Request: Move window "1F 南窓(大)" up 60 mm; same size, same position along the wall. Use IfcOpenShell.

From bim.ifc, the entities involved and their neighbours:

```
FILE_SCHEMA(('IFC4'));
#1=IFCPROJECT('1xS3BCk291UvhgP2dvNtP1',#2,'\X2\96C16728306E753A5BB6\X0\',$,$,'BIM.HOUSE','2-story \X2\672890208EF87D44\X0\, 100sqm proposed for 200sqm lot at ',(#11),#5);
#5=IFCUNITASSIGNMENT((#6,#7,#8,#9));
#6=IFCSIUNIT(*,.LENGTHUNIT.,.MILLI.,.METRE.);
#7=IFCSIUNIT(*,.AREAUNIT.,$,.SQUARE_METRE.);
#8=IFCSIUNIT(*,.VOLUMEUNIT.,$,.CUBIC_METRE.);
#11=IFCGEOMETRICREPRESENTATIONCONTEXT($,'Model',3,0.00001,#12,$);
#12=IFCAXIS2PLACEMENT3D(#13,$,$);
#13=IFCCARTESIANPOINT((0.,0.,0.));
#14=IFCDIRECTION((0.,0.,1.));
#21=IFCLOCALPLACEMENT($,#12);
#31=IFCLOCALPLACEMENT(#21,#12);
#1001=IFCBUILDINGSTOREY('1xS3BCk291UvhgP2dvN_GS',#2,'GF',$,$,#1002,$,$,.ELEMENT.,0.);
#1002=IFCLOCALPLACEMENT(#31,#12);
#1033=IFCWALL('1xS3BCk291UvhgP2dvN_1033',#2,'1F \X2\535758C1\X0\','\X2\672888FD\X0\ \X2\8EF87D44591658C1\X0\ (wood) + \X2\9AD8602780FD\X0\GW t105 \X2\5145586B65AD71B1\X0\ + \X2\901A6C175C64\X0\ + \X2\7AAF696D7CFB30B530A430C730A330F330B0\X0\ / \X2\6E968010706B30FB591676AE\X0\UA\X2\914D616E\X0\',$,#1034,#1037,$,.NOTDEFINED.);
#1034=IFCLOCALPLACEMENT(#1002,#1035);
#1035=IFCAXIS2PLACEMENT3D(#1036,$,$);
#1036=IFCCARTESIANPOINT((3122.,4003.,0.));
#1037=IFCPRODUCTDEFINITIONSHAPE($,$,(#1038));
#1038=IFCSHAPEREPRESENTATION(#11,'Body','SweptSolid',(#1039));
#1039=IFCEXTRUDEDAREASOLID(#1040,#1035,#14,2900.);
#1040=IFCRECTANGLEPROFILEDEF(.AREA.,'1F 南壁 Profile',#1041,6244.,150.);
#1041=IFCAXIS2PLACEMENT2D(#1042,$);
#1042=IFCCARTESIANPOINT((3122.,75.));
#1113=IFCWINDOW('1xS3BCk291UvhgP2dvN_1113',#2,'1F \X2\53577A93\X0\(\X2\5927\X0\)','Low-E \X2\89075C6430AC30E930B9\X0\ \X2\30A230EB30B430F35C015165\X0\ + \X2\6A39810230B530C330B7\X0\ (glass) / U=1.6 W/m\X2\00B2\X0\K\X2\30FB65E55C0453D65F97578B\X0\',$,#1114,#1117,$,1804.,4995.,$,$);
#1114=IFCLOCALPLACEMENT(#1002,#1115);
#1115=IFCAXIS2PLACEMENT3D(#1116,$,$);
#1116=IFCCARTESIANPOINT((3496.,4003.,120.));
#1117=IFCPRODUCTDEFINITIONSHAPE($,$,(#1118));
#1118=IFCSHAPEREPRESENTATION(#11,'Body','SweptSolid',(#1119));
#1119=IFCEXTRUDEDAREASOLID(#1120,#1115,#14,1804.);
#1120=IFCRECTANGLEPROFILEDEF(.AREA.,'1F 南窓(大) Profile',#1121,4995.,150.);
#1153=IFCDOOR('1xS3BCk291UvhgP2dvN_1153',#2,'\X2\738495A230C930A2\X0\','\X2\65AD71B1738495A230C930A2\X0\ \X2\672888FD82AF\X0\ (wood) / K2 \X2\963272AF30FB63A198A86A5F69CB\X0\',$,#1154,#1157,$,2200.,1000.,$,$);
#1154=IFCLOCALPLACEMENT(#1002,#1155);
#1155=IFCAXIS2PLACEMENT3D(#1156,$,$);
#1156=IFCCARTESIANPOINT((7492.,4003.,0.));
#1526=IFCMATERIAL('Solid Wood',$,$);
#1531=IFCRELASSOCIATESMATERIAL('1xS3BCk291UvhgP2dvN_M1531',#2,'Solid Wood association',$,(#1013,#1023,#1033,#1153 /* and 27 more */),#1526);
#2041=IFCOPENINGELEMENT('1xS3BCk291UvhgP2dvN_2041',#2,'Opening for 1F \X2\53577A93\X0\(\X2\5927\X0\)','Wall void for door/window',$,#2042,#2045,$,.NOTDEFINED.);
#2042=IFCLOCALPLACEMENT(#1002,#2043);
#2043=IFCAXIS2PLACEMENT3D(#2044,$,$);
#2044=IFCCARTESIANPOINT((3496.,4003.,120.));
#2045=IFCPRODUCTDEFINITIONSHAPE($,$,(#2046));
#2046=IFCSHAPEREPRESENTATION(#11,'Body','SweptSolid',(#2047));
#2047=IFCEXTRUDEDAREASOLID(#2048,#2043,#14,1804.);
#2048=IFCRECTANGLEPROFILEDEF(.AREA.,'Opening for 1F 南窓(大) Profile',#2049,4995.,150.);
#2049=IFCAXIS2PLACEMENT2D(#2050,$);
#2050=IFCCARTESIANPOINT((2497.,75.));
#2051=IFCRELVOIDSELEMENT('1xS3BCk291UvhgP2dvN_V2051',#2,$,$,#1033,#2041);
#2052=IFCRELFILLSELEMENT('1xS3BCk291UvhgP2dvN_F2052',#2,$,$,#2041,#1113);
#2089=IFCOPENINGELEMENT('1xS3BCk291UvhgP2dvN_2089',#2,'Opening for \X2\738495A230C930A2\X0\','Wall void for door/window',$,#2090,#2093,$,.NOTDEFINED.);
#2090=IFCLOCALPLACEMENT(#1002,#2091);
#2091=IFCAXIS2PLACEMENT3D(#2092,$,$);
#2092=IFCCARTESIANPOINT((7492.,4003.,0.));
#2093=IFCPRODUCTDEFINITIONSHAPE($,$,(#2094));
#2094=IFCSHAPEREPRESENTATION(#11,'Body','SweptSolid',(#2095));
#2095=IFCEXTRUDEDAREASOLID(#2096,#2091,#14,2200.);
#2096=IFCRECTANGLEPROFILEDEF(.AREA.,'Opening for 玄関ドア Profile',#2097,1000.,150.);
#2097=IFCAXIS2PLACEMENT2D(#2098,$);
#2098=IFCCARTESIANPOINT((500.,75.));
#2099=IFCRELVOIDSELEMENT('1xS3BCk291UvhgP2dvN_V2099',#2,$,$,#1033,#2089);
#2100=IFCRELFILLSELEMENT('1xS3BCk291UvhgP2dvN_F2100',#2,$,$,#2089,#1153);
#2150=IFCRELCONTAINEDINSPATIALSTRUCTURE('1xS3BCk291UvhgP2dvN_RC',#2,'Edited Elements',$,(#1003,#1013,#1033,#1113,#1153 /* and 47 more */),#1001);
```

```python
import numpy as np
import ifcopenshell
import ifcopenshell.api.geometry
import ifcopenshell.util.placement
import ifcopenshell.util.unit

model = ifcopenshell.open("bim.ifc")
unit_scale = ifcopenshell.util.unit.calculate_unit_scale(model)

window = model.by_id(1113)
opening = window.FillsVoids[0].RelatingOpeningElement
dz = 60.0

shift = np.array([0.0, 0.0, dz])
# The window is not placed relative to its opening, so move both.
for product in (opening, window):
    matrix = ifcopenshell.util.placement.get_local_placement(product.ObjectPlacement)
    matrix[:3, 3] += shift
    ifcopenshell.api.geometry.edit_object_placement(model, product=product, matrix=matrix, is_si=False)

print(f"moved by {dz * unit_scale:+.3f} m")

model.write("bim-out.ifc")
```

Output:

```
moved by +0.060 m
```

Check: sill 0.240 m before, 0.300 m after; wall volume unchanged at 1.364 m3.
